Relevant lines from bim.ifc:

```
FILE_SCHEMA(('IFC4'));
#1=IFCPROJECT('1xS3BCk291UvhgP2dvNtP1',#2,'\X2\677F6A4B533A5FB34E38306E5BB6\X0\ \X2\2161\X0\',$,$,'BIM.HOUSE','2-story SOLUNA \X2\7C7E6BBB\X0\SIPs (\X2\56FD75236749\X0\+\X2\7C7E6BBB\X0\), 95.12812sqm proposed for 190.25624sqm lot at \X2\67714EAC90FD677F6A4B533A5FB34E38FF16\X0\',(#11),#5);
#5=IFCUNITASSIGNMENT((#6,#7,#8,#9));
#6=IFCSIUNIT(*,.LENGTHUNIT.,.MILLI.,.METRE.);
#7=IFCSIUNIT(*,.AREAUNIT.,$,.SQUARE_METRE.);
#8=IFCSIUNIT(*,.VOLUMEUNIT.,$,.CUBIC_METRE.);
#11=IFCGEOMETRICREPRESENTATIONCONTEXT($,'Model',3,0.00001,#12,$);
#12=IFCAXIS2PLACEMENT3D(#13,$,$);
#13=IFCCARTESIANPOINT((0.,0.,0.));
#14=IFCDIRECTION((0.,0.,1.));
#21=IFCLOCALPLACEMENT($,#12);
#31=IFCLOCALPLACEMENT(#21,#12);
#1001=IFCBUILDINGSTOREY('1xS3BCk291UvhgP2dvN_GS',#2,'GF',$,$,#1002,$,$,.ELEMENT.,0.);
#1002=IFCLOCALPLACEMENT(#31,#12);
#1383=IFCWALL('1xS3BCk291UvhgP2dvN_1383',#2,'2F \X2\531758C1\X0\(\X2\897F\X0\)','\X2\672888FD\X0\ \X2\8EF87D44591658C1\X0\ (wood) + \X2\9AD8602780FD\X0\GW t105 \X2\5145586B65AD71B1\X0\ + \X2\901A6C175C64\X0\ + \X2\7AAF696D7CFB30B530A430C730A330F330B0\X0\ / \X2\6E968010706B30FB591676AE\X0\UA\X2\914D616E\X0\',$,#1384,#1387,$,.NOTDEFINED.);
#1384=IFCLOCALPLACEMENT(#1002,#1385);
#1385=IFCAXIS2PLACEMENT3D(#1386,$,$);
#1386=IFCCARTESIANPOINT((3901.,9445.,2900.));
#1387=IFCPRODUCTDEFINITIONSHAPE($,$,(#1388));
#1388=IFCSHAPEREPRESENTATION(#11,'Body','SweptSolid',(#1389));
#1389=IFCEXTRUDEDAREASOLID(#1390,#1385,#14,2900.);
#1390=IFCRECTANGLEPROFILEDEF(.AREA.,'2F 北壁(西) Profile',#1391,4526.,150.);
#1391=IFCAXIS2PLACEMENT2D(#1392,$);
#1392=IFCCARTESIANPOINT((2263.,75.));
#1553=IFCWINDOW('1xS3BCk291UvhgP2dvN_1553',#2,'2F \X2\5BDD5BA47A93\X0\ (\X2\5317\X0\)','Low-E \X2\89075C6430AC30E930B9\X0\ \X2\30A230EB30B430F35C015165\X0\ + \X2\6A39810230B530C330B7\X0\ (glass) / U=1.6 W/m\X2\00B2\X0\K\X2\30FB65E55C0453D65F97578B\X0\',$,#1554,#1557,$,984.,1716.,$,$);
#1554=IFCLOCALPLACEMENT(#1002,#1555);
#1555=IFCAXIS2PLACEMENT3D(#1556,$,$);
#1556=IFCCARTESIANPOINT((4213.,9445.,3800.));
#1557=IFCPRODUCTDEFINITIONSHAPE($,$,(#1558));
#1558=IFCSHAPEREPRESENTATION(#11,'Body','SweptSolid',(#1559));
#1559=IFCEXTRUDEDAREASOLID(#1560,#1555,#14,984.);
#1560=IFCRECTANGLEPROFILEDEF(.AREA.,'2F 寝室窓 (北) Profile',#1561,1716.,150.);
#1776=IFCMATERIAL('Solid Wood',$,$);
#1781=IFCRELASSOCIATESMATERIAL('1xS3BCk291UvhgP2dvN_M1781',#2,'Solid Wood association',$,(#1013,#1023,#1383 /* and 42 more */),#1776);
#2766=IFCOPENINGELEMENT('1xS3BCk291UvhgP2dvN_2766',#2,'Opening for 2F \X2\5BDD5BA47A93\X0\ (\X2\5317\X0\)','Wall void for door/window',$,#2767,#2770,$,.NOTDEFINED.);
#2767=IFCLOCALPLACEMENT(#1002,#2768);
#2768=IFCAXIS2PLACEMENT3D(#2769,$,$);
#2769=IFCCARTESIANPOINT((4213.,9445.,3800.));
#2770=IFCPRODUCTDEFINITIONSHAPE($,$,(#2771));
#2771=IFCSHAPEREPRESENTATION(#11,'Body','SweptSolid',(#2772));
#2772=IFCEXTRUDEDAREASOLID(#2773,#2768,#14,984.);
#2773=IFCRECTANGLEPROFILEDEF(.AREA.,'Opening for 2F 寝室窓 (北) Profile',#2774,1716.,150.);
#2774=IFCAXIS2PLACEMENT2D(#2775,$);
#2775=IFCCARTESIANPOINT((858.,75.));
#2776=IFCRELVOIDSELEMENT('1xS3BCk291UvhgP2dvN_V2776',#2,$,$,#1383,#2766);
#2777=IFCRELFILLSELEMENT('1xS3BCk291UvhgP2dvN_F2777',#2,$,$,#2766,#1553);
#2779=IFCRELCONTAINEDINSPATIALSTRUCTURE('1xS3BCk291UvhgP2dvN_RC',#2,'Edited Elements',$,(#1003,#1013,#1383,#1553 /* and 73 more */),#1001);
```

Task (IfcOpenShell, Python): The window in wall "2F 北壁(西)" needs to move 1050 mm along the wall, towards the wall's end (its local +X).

```python
import ifcopenshell
import ifcopenshell.api.geometry
import ifcopenshell.util.placement

model = ifcopenshell.open("bim.ifc")

window = model.by_guid("1xS3BCk291UvhgP2dvN_1553")
opening = window.FillsVoids[0].RelatingOpeningElement
wall = opening.VoidsElements[0].RelatingBuildingElement

wall_matrix = ifcopenshell.util.placement.get_local_placement(wall.ObjectPlacement)
shift = wall_matrix[:3, 0] * 1050.0
before = ifcopenshell.util.placement.get_local_placement(window.ObjectPlacement)[:3, 3].copy()

# The window is not placed relative to its opening, so move both.
for product in (opening, window):
    matrix = ifcopenshell.util.placement.get_local_placement(product.ObjectPlacement)
    matrix[:3, 3] += shift
    ifcopenshell.api.geometry.edit_object_placement(model, product=product, matrix=matrix, is_si=False)

after = ifcopenshell.util.placement.get_local_placement(window.ObjectPlacement)[:3, 3]
print("window moved by", (after - before).round(3) + 0.0)

model.write("bim_v2.ifc")
```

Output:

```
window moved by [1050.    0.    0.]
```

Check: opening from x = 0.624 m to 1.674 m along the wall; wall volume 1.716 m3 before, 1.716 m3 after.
